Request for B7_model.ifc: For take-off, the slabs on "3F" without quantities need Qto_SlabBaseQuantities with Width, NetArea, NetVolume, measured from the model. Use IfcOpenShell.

First a look at what the model holds.

```python
import ifcopenshell
import ifcopenshell.util.element
import ifcopenshell.util.unit

model = ifcopenshell.open("B7_model.ifc")
print(model.schema)
for unit_type in ("LENGTHUNIT", "AREAUNIT", "VOLUMEUNIT"):
    print(unit_type, ifcopenshell.util.unit.calculate_unit_scale(model, unit_type))
storey = next(s for s in model.by_type("IfcBuildingStorey") if s.Name == "3F")
slabs = [e for e in ifcopenshell.util.element.get_decomposition(storey) if e.is_a("IfcSlab")]
for e in sorted(slabs, key=lambda e: e.id()):
    print(e.id(), e.is_a(), e.Name, list(ifcopenshell.util.element.get_psets(e, qtos_only=True)), sep=" | ")
```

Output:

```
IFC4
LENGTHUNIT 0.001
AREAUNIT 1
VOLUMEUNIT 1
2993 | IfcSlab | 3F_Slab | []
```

```python
import ifcopenshell
import ifcopenshell.api.pset
import ifcopenshell.geom
import ifcopenshell.util.element
import ifcopenshell.util.shape
import ifcopenshell.util.unit

model = ifcopenshell.open("B7_model.ifc")
unit_scale = ifcopenshell.util.unit.calculate_unit_scale(model)
area_scale = ifcopenshell.util.unit.calculate_unit_scale(model, "AREAUNIT")
volume_scale = ifcopenshell.util.unit.calculate_unit_scale(model, "VOLUMEUNIT")
settings = ifcopenshell.geom.settings()

storey = next(s for s in model.by_type("IfcBuildingStorey") if s.Name == "3F")
slabs = [e for e in ifcopenshell.util.element.get_decomposition(storey) if e.is_a("IfcSlab")]

for e in sorted(slabs, key=lambda e: e.id()):
    if ifcopenshell.util.element.get_psets(e, qtos_only=True, should_inherit=False):
        continue
    # Geometry comes back in metres, in the element's own axes.
    shape = ifcopenshell.geom.create_shape(settings, e)
    values = {
        "Width": ifcopenshell.util.shape.get_z(shape.geometry) / unit_scale,
        "NetArea": ifcopenshell.util.shape.get_footprint_area(shape.geometry) / area_scale,
        "NetVolume": ifcopenshell.util.shape.get_volume(shape.geometry) / volume_scale,
    }
    qto = ifcopenshell.api.pset.add_qto(model, product=e, name="Qto_SlabBaseQuantities")
    ifcopenshell.api.pset.edit_qto(model, qto=qto, properties=values)
    print(e.id(), {k: round(v, 3) for k, v in values.items()})

model.write("B7_model_updated.ifc")
```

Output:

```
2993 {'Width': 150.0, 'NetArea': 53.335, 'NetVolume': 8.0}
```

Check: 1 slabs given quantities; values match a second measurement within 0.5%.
